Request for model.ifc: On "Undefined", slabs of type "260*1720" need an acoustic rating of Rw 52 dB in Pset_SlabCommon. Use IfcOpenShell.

First a look at what the model holds.

```python
import ifcopenshell
import ifcopenshell.util.element

model = ifcopenshell.open("model.ifc")
print(model.schema)
storey = next(s for s in model.by_type("IfcBuildingStorey") if s.Name == "Undefined")
slabs = [e for e in ifcopenshell.util.element.get_decomposition(storey) if e.is_a("IfcSlab")]
seen = {}
for e in slabs:
    element_type = ifcopenshell.util.element.get_type(e)
    key = (element_type.Name if element_type != e and element_type else None, ifcopenshell.util.element.get_pset(e, "Pset_SlabCommon", "AcousticRating"))
    seen[key] = seen.get(key, 0) + 1
for (name, value), count in sorted(seen.items(), key=str):
    print(count, "x", name, "|", value)
```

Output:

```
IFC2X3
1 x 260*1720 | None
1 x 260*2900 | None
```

```python
import ifcopenshell
import ifcopenshell.api.pset
import ifcopenshell.util.element

model = ifcopenshell.open("model.ifc")

storey = next(s for s in model.by_type("IfcBuildingStorey") if s.Name == "Undefined")
slabs = [e for e in ifcopenshell.util.element.get_decomposition(storey) if e.is_a("IfcSlab")]

count = 0
for e in slabs:
    element_type = ifcopenshell.util.element.get_type(e)
    if element_type in (None, e) or element_type.Name != "260*1720":
        continue
    # add_pset returns the element's existing set when there is one.
    pset = ifcopenshell.api.pset.add_pset(model, product=e, name="Pset_SlabCommon")
    ifcopenshell.api.pset.edit_pset(model, pset=pset, properties={"AcousticRating": "Rw 52 dB"})
    count += 1

print(count, "slabs updated")

model.write("model_edited.ifc")
```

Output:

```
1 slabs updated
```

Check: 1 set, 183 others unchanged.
